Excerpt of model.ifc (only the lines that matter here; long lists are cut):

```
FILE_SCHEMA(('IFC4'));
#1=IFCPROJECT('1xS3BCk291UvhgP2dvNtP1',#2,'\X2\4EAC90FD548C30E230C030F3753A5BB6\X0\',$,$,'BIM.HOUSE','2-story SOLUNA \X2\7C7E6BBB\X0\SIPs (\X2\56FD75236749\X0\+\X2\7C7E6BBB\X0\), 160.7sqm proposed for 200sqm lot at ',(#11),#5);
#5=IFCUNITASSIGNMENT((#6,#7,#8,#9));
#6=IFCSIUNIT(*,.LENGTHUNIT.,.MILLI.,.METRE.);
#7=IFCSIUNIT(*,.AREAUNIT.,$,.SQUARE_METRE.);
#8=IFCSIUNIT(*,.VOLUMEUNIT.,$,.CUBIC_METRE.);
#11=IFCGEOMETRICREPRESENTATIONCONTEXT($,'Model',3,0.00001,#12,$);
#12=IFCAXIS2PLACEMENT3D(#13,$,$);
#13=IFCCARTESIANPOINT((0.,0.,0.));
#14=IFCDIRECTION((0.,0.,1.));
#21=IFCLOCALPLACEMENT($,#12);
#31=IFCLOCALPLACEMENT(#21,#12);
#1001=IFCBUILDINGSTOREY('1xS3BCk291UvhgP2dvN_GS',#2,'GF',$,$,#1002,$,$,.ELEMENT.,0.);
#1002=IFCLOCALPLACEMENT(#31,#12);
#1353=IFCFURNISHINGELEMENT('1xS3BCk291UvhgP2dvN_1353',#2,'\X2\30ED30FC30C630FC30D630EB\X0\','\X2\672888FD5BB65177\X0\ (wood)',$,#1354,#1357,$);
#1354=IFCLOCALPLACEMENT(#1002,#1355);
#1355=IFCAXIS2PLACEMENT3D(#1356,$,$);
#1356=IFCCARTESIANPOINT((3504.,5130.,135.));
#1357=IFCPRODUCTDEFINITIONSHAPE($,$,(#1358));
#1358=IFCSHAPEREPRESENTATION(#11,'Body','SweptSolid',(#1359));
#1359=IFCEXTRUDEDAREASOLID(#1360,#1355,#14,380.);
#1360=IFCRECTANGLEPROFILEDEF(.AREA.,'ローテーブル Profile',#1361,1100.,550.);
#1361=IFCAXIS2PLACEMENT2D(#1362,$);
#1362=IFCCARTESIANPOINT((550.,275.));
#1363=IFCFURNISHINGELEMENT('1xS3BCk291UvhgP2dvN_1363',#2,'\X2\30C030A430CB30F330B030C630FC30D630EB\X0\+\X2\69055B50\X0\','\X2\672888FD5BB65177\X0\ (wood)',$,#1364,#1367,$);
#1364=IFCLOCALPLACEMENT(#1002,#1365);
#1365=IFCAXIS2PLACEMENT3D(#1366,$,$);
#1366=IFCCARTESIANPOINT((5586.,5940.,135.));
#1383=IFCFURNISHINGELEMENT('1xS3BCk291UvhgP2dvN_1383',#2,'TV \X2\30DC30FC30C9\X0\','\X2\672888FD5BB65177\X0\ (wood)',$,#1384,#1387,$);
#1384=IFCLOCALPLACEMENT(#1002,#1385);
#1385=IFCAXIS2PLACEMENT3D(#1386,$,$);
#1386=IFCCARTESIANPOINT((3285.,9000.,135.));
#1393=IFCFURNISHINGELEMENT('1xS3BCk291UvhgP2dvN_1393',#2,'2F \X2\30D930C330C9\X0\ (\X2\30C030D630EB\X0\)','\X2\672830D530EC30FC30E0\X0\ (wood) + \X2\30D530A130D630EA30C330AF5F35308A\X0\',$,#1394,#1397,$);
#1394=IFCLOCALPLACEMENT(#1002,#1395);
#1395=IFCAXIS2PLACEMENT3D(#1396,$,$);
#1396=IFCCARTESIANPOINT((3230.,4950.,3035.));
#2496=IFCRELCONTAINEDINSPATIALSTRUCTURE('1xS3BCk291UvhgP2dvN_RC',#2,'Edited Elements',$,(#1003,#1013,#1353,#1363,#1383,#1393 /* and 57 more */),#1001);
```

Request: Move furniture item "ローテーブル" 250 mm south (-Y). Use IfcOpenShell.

```python
import ifcopenshell
import ifcopenshell.api.geometry
import ifcopenshell.util.placement
import ifcopenshell.util.unit

model = ifcopenshell.open("model.ifc")
unit_scale = ifcopenshell.util.unit.calculate_unit_scale(model)

item = model.by_id(1353)
matrix = ifcopenshell.util.placement.get_local_placement(item.ObjectPlacement)
matrix[1, 3] -= 0.25 / unit_scale
ifcopenshell.api.geometry.edit_object_placement(model, product=item, matrix=matrix, is_si=False)

print(ifcopenshell.util.placement.get_local_placement(item.ObjectPlacement).round(3) + 0.0)

model.write("model_updated.ifc")
```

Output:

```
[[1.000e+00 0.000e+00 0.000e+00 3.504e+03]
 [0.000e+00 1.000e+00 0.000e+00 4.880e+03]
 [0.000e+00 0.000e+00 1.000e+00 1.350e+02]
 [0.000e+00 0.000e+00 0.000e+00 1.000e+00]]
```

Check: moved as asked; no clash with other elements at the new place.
